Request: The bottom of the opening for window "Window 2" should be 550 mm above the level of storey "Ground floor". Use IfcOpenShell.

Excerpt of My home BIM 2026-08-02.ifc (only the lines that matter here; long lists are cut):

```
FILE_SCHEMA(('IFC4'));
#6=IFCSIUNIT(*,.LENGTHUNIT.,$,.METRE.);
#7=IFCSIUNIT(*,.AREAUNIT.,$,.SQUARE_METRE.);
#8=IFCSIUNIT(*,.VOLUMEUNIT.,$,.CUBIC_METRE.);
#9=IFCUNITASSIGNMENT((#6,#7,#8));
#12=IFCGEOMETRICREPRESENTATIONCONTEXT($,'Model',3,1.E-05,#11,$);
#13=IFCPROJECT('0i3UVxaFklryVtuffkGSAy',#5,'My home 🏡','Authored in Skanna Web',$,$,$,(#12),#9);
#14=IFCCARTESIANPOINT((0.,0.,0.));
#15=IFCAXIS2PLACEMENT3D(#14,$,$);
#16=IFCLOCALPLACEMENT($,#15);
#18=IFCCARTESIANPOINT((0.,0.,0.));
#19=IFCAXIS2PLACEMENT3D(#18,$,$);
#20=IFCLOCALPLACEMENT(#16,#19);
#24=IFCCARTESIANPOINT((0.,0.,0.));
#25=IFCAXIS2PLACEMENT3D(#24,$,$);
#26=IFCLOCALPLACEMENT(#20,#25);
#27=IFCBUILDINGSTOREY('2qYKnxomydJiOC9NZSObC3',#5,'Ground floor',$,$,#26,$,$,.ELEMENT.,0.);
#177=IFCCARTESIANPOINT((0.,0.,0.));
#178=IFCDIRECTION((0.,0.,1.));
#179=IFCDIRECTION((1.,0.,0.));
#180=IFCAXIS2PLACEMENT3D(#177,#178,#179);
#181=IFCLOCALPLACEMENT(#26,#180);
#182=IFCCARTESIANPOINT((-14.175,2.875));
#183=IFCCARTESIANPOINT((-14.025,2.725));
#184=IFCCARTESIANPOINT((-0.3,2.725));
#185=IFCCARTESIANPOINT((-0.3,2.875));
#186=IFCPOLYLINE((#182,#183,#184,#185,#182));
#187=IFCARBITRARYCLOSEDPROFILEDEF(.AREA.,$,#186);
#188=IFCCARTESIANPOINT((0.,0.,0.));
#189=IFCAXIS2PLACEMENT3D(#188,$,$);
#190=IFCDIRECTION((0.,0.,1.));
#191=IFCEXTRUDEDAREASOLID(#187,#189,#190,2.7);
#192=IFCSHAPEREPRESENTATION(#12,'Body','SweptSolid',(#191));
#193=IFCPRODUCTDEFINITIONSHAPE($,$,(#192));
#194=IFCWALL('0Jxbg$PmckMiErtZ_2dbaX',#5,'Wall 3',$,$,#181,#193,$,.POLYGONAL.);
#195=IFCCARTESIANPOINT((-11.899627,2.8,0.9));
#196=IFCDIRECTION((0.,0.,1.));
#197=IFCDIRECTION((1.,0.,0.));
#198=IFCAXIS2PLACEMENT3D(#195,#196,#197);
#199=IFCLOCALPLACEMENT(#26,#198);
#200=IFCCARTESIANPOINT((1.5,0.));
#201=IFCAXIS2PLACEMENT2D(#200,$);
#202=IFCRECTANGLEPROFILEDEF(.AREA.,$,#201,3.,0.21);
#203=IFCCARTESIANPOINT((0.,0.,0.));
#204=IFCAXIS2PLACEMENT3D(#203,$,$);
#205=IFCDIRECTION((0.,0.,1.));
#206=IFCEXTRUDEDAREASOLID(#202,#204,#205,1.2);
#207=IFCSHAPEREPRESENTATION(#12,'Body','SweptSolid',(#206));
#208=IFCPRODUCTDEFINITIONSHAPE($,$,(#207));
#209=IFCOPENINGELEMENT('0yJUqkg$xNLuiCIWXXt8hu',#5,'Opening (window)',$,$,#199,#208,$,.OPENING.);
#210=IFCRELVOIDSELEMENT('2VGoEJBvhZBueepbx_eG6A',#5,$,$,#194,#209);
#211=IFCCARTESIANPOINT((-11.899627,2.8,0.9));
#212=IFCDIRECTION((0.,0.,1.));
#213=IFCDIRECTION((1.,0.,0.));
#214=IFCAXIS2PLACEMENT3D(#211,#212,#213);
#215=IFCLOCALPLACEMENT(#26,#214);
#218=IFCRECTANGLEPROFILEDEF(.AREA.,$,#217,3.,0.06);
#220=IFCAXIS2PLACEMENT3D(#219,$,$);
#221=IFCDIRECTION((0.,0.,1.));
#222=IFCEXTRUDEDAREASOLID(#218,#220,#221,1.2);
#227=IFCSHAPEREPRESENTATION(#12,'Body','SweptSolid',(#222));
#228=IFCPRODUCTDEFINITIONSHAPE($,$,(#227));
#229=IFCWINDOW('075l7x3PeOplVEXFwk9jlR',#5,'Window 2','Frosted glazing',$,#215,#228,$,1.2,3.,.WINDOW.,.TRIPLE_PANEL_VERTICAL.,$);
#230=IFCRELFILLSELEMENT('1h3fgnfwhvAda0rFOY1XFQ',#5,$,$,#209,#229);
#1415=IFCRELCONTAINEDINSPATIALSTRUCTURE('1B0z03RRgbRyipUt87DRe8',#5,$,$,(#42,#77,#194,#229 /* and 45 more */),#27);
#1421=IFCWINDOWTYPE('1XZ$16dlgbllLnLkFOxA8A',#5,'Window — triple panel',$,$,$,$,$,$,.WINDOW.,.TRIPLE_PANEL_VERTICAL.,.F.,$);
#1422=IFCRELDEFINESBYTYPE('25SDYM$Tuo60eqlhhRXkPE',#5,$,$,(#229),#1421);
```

```python
import numpy as np
import ifcopenshell
import ifcopenshell.api.geometry
import ifcopenshell.geom
import ifcopenshell.util.element
import ifcopenshell.util.placement
import ifcopenshell.util.shape
import ifcopenshell.util.unit

model = ifcopenshell.open("My home BIM 2026-08-02.ifc")
unit_scale = ifcopenshell.util.unit.calculate_unit_scale(model)

window = model.by_guid("075l7x3PeOplVEXFwk9jlR")
opening = window.FillsVoids[0].RelatingOpeningElement
storey = ifcopenshell.util.element.get_container(window, ifc_class="IfcBuildingStorey")
level = ifcopenshell.util.placement.get_local_placement(storey.ObjectPlacement)[2, 3]

# The opening's origin need not be at the sill, so measure its lowest point.
shape = ifcopenshell.geom.create_shape(ifcopenshell.geom.settings(), opening)
bottom = ifcopenshell.util.shape.get_shape_bottom_elevation(shape, shape.geometry) / unit_scale
dz = level + 0.55 - bottom

shift = np.array([0.0, 0.0, dz])
# The window is not placed relative to its opening, so move both.
for product in (opening, window):
    matrix = ifcopenshell.util.placement.get_local_placement(product.ObjectPlacement)
    matrix[:3, 3] += shift
    ifcopenshell.api.geometry.edit_object_placement(model, product=product, matrix=matrix, is_si=False)

print(f"moved by {dz * unit_scale:+.3f} m")

model.write("My home BIM 2026-08-02_rev.ifc")
```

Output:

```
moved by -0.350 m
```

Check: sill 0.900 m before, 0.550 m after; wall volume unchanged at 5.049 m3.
